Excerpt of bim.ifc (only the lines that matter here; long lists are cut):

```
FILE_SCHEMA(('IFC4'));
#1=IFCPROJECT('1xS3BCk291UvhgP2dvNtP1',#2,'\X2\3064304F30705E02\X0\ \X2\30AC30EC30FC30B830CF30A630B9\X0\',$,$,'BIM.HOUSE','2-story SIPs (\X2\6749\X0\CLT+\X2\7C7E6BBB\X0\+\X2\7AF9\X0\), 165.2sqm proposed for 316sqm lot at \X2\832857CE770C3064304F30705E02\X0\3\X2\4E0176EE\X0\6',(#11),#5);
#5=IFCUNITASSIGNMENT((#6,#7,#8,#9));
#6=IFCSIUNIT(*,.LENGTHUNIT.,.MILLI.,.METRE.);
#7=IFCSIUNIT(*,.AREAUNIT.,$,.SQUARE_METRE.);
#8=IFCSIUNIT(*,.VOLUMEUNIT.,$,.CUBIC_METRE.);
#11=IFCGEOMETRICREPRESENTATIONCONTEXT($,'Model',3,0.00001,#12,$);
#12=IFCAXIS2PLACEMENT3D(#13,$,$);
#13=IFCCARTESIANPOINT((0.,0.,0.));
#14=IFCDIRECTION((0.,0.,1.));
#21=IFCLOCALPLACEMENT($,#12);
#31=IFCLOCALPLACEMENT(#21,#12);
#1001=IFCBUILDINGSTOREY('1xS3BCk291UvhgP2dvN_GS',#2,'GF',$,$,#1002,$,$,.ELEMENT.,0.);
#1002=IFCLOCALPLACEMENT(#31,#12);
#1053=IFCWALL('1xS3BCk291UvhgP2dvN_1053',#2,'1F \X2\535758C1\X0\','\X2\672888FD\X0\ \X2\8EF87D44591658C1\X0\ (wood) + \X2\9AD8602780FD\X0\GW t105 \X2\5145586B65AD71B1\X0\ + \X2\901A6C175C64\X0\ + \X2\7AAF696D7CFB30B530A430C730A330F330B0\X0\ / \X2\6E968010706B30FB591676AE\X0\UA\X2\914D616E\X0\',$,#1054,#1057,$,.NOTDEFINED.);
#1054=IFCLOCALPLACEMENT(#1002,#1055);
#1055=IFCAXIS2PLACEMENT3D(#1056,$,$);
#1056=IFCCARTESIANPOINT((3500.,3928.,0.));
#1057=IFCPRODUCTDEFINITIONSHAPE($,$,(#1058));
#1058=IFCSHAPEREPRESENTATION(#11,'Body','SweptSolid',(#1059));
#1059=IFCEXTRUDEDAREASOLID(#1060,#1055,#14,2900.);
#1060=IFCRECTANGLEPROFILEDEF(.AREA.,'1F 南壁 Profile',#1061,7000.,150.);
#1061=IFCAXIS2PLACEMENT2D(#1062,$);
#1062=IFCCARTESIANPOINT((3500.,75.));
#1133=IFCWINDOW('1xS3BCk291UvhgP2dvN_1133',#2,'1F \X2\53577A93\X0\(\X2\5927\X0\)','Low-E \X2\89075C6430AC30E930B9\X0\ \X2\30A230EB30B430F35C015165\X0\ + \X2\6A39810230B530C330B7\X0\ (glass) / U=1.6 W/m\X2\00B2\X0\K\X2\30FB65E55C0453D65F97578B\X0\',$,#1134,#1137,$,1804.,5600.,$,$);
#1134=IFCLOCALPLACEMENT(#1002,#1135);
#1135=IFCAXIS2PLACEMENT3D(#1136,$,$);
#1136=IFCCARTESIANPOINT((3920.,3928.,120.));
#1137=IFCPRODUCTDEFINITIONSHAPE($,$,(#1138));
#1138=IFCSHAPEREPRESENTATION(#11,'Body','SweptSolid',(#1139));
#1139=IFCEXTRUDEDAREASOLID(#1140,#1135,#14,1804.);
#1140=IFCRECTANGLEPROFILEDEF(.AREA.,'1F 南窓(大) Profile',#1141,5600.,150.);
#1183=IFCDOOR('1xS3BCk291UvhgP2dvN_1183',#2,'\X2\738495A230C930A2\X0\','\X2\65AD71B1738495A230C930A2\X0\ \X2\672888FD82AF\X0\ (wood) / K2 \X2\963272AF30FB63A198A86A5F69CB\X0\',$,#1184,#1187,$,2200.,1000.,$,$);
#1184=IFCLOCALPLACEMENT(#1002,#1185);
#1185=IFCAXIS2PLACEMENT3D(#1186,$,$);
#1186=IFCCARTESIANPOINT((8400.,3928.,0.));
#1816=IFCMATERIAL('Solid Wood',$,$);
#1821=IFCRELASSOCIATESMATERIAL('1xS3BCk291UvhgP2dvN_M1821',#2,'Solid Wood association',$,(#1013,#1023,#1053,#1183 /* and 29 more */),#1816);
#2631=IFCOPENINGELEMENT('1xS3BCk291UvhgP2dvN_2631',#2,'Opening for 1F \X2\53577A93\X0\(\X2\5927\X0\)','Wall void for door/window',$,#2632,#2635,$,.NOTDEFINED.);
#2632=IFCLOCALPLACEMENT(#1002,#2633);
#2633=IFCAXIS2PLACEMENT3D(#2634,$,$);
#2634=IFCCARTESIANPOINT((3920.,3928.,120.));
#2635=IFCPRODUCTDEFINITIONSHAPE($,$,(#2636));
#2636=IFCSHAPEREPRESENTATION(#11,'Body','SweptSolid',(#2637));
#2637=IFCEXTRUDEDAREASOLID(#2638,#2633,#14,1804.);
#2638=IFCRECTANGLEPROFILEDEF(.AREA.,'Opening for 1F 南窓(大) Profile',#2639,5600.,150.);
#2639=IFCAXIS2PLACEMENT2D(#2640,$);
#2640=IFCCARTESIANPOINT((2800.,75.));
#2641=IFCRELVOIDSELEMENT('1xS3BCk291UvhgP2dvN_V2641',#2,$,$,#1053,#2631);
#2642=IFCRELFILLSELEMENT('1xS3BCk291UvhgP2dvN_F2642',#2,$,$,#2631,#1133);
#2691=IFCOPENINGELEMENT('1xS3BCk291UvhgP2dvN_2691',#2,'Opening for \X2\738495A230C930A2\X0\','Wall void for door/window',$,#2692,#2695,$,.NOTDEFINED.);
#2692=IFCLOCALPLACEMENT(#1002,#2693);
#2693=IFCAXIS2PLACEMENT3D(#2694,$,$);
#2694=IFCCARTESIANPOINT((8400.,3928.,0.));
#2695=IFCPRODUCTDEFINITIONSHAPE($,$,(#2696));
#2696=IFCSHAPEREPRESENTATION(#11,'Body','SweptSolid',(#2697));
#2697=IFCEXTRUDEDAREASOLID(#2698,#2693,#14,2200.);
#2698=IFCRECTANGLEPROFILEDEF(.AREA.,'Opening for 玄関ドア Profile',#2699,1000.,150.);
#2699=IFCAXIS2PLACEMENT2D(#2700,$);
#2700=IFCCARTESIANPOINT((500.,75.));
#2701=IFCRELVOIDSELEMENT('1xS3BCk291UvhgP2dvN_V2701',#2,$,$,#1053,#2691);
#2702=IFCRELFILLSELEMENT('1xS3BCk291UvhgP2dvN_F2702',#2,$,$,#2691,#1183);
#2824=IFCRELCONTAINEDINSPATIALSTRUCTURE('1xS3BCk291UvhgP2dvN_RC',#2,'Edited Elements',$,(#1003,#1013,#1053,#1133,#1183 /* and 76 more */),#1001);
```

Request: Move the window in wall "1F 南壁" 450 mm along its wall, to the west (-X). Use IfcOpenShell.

```python
import ifcopenshell
import ifcopenshell.api.geometry
import ifcopenshell.util.placement

model = ifcopenshell.open("bim.ifc")

window = model.by_id(1133)
opening = window.FillsVoids[0].RelatingOpeningElement
wall = opening.VoidsElements[0].RelatingBuildingElement

wall_matrix = ifcopenshell.util.placement.get_local_placement(wall.ObjectPlacement)
shift = wall_matrix[:3, 0] * -450.0
before = ifcopenshell.util.placement.get_local_placement(window.ObjectPlacement)[:3, 3].copy()

# The window is not placed relative to its opening, so move both.
for product in (opening, window):
    matrix = ifcopenshell.util.placement.get_local_placement(product.ObjectPlacement)
    matrix[:3, 3] += shift
    ifcopenshell.api.geometry.edit_object_placement(model, product=product, matrix=matrix, is_si=False)

after = ifcopenshell.util.placement.get_local_placement(window.ObjectPlacement)[:3, 3]
print("window moved by", (after - before).round(3) + 0.0)

model.write("bim_rev.ifc")
```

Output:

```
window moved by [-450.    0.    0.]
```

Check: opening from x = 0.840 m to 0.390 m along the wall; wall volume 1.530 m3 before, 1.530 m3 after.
